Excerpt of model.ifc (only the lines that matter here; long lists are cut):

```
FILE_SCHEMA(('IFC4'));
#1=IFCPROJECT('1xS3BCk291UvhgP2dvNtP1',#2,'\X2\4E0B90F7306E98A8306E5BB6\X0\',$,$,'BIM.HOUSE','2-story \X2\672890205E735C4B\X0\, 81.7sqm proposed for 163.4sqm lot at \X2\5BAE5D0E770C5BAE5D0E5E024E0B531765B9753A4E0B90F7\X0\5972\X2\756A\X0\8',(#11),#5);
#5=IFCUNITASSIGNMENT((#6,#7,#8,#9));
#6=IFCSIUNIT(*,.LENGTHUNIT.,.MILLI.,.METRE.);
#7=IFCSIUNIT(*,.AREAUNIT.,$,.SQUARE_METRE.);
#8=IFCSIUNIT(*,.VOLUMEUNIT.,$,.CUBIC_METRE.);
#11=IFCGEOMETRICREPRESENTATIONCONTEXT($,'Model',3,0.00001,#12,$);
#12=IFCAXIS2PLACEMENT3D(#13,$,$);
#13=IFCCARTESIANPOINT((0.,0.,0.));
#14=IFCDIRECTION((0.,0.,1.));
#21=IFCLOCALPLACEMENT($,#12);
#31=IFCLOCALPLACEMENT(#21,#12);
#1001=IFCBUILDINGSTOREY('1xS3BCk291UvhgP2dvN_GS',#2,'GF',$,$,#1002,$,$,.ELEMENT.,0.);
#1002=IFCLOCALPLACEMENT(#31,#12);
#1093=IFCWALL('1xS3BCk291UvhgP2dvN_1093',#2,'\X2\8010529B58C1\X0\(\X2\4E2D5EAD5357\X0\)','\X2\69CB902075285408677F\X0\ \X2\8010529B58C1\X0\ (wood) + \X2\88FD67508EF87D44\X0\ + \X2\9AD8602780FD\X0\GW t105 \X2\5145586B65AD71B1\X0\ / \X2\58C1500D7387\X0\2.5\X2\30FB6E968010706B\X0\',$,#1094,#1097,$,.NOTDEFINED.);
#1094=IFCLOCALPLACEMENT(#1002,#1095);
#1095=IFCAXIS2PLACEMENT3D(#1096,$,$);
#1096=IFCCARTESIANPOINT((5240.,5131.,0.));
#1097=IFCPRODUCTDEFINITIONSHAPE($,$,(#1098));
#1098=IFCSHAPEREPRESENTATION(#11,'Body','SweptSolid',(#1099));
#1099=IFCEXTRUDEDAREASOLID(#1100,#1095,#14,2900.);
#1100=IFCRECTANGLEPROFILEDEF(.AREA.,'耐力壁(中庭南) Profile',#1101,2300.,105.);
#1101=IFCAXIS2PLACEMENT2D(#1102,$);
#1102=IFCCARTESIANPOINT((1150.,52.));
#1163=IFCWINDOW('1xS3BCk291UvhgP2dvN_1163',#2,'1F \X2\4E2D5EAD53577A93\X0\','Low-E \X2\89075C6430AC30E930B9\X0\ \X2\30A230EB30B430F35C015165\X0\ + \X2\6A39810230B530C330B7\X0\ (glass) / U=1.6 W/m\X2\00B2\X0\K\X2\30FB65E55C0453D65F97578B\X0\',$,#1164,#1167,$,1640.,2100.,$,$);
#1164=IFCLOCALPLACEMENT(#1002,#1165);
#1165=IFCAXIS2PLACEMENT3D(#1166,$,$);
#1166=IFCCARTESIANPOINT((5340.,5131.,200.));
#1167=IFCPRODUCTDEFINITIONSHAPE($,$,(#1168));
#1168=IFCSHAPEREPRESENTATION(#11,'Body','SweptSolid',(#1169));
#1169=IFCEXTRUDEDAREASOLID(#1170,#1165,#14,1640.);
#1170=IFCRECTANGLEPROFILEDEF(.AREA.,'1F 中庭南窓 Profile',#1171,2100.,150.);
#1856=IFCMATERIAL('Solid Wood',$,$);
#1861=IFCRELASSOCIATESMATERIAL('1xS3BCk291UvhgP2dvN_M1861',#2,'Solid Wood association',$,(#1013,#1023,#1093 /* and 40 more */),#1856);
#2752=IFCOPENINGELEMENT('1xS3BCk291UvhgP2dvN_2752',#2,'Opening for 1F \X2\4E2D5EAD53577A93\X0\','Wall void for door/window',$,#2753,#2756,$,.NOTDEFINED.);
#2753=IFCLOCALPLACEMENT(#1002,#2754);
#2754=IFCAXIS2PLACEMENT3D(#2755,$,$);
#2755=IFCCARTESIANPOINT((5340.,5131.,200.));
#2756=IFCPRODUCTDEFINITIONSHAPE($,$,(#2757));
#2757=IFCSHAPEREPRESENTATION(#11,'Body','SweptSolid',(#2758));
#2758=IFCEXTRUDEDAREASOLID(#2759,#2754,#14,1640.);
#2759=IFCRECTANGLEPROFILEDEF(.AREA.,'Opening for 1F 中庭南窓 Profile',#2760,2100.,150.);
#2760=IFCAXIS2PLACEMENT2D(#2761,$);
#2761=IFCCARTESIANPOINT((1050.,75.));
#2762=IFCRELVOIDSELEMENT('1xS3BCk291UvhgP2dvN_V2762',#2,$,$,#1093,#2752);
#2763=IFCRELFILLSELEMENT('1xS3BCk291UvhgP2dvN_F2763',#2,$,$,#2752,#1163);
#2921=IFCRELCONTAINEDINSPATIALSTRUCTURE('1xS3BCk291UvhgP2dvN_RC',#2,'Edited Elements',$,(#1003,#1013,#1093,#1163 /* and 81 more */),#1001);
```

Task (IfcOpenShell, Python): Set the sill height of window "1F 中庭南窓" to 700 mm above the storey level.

```python
import numpy as np
import ifcopenshell
import ifcopenshell.api.geometry
import ifcopenshell.geom
import ifcopenshell.util.element
import ifcopenshell.util.placement
import ifcopenshell.util.shape
import ifcopenshell.util.unit

model = ifcopenshell.open("model.ifc")
unit_scale = ifcopenshell.util.unit.calculate_unit_scale(model)

window = model.by_id(1163)
opening = window.FillsVoids[0].RelatingOpeningElement
storey = ifcopenshell.util.element.get_container(window, ifc_class="IfcBuildingStorey")
level = ifcopenshell.util.placement.get_local_placement(storey.ObjectPlacement)[2, 3]

# The opening's origin need not be at the sill, so measure its lowest point.
shape = ifcopenshell.geom.create_shape(ifcopenshell.geom.settings(), opening)
bottom = ifcopenshell.util.shape.get_shape_bottom_elevation(shape, shape.geometry) / unit_scale
dz = level + 0.7 / unit_scale - bottom

shift = np.array([0.0, 0.0, dz])
# The window is not placed relative to its opening, so move both.
for product in (opening, window):
    matrix = ifcopenshell.util.placement.get_local_placement(product.ObjectPlacement)
    matrix[:3, 3] += shift
    ifcopenshell.api.geometry.edit_object_placement(model, product=product, matrix=matrix, is_si=False)

print(f"moved by {dz * unit_scale:+.3f} m")

model.write("model_edited.ifc")
```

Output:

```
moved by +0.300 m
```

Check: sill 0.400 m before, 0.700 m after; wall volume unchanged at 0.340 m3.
